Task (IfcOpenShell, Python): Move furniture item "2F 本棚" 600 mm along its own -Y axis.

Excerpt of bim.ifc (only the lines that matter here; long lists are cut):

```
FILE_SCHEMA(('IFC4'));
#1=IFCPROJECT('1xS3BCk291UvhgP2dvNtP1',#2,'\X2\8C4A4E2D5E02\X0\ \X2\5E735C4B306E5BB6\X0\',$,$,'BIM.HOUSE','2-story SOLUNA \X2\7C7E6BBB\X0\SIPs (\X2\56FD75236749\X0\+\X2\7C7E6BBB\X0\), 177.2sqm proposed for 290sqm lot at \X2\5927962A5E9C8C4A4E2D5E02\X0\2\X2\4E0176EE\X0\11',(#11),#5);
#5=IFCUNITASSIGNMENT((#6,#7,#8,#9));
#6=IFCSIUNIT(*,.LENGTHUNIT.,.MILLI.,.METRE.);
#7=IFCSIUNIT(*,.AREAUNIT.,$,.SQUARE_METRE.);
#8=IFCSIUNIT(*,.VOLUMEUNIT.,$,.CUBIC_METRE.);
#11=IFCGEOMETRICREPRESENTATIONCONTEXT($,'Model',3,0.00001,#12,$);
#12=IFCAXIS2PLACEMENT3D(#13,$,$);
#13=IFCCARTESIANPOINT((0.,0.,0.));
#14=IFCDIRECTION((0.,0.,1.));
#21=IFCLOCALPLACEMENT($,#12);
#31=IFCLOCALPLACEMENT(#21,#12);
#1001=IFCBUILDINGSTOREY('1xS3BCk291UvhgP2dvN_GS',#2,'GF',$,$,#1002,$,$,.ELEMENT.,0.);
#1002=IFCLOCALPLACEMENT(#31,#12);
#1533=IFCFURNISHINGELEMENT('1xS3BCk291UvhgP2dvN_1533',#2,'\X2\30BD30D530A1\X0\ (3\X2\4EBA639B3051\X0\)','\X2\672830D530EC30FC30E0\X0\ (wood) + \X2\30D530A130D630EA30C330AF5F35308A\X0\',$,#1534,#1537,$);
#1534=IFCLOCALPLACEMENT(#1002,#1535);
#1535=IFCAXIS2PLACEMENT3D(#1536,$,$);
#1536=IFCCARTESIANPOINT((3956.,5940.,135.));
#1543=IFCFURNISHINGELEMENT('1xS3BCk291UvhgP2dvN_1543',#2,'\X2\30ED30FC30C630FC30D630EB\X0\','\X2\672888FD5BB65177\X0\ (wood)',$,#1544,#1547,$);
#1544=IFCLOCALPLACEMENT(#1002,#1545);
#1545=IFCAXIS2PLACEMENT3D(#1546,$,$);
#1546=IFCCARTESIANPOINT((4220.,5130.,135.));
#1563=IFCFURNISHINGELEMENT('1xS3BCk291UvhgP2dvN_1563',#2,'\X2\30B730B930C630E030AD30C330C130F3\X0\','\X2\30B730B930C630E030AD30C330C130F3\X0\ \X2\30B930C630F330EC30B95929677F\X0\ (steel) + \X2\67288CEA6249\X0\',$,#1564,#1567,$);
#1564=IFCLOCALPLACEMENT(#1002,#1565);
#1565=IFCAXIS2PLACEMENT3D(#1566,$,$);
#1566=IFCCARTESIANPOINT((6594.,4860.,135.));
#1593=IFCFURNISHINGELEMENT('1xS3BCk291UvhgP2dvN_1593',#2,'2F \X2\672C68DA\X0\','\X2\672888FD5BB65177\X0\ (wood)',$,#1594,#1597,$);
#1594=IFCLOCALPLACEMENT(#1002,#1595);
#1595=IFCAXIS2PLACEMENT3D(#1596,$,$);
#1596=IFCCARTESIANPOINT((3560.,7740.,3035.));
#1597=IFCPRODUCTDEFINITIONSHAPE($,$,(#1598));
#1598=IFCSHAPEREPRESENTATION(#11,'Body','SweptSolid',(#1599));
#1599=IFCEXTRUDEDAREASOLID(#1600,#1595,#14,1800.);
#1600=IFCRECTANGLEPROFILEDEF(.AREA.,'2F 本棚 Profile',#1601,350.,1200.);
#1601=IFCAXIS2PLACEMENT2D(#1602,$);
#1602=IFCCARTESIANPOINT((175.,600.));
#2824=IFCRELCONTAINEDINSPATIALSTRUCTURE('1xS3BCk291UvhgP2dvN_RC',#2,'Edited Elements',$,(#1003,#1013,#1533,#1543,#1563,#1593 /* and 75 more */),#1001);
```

```python
import ifcopenshell
import ifcopenshell.api.geometry
import ifcopenshell.util.placement

model = ifcopenshell.open("bim.ifc")

item = model.by_guid("1xS3BCk291UvhgP2dvN_1593")
matrix = ifcopenshell.util.placement.get_local_placement(item.ObjectPlacement)
matrix[:3, 3] -= matrix[:3, 1] * 600.0
ifcopenshell.api.geometry.edit_object_placement(model, product=item, matrix=matrix, is_si=False)

print(ifcopenshell.util.placement.get_local_placement(item.ObjectPlacement).round(3) + 0.0)

model.write("bim-out.ifc")
```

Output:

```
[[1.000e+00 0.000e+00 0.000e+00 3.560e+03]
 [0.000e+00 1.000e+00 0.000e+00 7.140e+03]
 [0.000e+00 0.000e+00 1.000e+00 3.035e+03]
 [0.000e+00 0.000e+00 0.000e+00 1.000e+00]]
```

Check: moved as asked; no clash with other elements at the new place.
